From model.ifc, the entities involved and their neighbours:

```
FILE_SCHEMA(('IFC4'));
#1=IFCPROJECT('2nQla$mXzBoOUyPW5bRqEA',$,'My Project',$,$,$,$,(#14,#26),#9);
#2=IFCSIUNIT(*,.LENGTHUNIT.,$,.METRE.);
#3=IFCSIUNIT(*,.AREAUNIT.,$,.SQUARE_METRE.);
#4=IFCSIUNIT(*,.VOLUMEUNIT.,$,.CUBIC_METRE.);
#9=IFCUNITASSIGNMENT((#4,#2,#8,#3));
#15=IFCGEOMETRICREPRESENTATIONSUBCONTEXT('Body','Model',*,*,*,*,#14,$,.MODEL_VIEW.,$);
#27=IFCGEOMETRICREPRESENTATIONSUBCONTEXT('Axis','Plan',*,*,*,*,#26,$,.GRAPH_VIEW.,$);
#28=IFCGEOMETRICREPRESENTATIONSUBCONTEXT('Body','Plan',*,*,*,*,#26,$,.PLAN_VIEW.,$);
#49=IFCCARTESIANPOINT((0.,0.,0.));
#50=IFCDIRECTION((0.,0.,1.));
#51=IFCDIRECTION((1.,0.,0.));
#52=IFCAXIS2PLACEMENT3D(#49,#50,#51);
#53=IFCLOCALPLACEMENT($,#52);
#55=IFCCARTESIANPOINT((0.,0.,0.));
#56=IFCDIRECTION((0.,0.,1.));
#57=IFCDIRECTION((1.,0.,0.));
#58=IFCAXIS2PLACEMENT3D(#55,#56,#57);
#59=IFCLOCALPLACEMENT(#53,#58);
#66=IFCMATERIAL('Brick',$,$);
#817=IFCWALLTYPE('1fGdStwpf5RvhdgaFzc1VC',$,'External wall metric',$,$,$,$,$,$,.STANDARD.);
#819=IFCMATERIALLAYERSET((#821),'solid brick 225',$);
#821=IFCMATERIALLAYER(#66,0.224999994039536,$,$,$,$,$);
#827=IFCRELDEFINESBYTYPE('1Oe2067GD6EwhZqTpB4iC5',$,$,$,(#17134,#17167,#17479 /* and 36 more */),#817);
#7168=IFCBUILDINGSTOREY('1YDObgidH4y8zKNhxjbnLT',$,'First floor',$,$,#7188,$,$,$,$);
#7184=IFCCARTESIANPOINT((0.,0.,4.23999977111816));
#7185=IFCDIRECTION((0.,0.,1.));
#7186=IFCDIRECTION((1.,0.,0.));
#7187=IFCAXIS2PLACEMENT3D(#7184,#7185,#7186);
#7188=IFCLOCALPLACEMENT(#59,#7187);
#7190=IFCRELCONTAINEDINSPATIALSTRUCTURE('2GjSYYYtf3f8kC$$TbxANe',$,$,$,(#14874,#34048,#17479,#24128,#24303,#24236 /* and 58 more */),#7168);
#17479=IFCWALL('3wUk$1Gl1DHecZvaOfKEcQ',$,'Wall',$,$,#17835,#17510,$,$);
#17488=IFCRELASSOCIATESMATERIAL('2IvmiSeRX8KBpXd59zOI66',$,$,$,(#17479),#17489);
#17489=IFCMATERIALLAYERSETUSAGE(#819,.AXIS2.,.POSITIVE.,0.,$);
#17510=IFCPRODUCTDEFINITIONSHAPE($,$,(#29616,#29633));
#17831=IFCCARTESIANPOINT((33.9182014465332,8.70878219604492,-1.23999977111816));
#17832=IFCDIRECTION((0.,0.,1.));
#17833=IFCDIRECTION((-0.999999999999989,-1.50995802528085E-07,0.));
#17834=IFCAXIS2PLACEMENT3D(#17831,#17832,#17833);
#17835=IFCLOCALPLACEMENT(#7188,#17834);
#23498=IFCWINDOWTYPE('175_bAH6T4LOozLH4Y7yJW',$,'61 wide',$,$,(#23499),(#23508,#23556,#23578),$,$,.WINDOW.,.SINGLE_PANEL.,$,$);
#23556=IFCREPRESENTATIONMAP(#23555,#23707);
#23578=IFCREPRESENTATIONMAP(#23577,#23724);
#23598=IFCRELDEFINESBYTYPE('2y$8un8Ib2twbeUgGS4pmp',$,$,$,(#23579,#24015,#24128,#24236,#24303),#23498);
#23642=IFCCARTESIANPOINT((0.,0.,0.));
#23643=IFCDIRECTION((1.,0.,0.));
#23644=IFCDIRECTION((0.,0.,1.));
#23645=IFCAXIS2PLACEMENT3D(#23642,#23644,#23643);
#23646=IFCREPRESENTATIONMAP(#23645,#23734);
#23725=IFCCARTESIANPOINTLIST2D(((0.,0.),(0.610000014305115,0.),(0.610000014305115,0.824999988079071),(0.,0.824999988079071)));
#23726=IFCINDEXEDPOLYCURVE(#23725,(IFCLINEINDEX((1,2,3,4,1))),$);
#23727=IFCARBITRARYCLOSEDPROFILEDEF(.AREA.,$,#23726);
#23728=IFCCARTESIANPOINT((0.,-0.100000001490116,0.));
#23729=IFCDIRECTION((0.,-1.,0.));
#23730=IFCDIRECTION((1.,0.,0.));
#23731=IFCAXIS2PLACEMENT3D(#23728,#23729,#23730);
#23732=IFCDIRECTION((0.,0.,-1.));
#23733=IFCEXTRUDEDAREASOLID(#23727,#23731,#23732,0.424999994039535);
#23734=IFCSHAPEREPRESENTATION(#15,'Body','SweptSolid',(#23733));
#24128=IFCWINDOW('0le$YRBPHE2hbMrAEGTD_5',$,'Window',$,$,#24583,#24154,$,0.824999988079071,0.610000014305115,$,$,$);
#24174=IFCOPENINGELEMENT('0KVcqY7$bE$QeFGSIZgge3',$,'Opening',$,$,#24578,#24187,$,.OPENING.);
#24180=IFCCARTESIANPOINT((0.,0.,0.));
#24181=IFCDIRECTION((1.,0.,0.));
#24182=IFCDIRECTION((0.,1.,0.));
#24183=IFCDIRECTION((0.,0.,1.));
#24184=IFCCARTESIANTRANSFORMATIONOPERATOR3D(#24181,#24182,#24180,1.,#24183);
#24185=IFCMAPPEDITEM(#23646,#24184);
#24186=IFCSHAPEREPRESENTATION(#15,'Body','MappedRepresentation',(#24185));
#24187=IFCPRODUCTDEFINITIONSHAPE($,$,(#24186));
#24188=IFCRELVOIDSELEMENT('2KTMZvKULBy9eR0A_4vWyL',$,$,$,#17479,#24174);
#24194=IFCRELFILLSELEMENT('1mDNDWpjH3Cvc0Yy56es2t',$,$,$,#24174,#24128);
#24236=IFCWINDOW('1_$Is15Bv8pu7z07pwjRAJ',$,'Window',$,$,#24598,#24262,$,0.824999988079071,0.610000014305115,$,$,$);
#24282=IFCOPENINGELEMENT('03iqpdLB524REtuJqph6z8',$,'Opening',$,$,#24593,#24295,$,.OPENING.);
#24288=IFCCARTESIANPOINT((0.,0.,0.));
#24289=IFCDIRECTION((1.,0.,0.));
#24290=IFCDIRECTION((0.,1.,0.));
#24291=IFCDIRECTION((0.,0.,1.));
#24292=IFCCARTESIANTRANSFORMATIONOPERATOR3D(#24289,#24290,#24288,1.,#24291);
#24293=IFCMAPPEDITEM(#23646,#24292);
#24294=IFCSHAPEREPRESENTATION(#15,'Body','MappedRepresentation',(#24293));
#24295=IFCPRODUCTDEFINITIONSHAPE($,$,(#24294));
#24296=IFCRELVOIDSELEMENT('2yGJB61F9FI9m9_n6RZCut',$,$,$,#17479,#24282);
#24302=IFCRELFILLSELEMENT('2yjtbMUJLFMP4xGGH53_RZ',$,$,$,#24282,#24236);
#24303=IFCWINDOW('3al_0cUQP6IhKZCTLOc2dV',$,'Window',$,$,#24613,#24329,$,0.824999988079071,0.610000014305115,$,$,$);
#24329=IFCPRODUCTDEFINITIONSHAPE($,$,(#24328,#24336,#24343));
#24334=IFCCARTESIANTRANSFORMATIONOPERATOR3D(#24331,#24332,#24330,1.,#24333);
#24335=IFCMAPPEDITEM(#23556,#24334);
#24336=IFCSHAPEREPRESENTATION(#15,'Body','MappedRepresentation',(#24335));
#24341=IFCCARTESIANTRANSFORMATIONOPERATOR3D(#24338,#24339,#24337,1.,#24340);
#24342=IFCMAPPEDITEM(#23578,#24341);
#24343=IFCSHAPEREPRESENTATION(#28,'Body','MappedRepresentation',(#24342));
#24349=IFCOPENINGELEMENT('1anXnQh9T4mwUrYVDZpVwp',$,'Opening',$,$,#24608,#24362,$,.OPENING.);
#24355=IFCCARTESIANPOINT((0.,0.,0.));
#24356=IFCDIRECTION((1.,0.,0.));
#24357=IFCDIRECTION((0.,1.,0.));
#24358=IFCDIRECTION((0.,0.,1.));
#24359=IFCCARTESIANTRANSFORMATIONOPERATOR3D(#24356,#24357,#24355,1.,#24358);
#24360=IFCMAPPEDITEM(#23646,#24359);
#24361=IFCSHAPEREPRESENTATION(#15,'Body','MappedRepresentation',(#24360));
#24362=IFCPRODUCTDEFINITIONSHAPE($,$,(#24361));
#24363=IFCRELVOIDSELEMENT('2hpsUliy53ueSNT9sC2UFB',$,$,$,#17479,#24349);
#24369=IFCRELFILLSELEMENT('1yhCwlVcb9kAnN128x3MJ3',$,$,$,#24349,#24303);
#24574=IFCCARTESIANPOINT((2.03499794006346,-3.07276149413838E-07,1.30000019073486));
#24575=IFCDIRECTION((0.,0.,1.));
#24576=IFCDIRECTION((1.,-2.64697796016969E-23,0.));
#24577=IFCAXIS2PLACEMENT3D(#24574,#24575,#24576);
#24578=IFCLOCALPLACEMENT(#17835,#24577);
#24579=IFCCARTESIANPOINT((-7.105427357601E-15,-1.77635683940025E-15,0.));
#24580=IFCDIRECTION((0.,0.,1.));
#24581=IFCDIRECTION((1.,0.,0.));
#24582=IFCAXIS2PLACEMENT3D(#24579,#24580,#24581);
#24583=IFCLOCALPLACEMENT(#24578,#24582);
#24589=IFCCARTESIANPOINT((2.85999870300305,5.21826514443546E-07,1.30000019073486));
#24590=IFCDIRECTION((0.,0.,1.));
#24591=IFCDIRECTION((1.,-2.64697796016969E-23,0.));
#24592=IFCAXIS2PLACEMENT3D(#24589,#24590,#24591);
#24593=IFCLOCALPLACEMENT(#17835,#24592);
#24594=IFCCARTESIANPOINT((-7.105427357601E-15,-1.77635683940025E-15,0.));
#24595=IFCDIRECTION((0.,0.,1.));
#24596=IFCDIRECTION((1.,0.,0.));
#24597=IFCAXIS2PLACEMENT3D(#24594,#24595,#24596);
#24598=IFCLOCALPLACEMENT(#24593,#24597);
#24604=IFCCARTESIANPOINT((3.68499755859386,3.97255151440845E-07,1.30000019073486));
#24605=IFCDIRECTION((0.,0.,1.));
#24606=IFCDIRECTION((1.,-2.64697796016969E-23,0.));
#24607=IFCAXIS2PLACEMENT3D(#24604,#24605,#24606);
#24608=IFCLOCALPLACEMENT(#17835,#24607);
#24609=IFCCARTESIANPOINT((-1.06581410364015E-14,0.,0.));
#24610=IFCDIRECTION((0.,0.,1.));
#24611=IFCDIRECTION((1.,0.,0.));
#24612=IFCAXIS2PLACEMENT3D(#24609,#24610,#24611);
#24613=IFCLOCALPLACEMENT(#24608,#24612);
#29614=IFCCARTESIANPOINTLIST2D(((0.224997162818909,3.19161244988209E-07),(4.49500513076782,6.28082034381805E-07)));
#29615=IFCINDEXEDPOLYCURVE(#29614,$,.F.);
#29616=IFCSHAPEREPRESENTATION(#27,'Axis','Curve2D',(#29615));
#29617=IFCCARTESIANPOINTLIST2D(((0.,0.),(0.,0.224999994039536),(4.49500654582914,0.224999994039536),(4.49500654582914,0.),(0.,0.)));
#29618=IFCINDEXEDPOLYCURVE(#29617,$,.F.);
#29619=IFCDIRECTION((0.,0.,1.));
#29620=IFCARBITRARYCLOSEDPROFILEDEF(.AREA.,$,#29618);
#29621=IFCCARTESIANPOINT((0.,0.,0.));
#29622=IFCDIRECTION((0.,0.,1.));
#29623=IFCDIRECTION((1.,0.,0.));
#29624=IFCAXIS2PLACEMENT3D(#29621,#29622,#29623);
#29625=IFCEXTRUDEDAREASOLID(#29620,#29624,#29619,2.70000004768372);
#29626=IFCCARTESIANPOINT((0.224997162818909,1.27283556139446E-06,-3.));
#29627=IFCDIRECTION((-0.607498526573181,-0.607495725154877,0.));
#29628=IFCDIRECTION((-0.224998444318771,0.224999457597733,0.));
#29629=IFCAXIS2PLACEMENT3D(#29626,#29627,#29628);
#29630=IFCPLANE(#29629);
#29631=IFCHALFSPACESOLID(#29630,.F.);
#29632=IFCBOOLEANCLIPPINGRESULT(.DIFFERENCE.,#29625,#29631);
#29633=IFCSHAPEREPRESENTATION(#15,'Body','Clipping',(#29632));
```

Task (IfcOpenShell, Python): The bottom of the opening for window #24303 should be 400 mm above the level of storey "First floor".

```python
import numpy as np
import ifcopenshell
import ifcopenshell.api.geometry
import ifcopenshell.geom
import ifcopenshell.util.element
import ifcopenshell.util.placement
import ifcopenshell.util.shape
import ifcopenshell.util.unit

model = ifcopenshell.open("model.ifc")
unit_scale = ifcopenshell.util.unit.calculate_unit_scale(model)

window = model.by_id(24303)
opening = window.FillsVoids[0].RelatingOpeningElement
storey = ifcopenshell.util.element.get_container(window, ifc_class="IfcBuildingStorey")
level = ifcopenshell.util.placement.get_local_placement(storey.ObjectPlacement)[2, 3]

# The opening's origin need not be at the sill, so measure its lowest point.
shape = ifcopenshell.geom.create_shape(ifcopenshell.geom.settings(), opening)
bottom = ifcopenshell.util.shape.get_shape_bottom_elevation(shape, shape.geometry) / unit_scale
dz = level + 0.4 - bottom

shift = np.array([0.0, 0.0, dz])
# The window is placed relative to its opening, so it follows when the opening moves.
matrix = ifcopenshell.util.placement.get_local_placement(opening.ObjectPlacement)
matrix[:3, 3] += shift
ifcopenshell.api.geometry.edit_object_placement(
    model, product=opening, matrix=matrix, is_si=False, should_transform_children=True
)

print(f"moved by {dz * unit_scale:+.3f} m")

model.write("model_v2.ifc")
```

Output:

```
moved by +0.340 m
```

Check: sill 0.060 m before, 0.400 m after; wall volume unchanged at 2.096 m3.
